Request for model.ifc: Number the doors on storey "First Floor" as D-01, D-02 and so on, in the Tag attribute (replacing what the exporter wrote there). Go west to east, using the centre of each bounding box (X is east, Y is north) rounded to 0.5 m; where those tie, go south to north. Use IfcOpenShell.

First a look at what the model holds.

```python
import ifcopenshell
import ifcopenshell.util.element
import ifcopenshell.util.placement

model = ifcopenshell.open("model.ifc")
print(model.schema)
storey = next(s for s in model.by_type("IfcBuildingStorey") if s.Name == "First Floor")
doors = [e for e in ifcopenshell.util.element.get_decomposition(storey) if e.is_a("IfcDoor")]
for e in sorted(doors, key=lambda e: e.id()):
    origin = ifcopenshell.util.placement.get_local_placement(e.ObjectPlacement)[:3, 3]
    print(e.id(), e.Tag, e.Name, origin.round(2) + 0.0, sep=" | ")
```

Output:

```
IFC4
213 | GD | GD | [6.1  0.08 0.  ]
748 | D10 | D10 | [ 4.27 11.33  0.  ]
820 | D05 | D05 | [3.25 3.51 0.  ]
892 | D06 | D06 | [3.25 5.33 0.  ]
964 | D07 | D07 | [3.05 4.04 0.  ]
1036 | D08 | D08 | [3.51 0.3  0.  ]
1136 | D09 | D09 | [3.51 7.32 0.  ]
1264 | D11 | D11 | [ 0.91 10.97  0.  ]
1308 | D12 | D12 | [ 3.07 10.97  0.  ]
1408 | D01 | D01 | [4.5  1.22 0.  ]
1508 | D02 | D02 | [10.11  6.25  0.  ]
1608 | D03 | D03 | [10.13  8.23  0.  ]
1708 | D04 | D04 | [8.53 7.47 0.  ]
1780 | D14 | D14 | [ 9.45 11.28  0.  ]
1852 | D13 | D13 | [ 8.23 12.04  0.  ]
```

```python
import ifcopenshell
import ifcopenshell.geom
import ifcopenshell.util.element
import ifcopenshell.util.shape

model = ifcopenshell.open("model.ifc")
settings = ifcopenshell.geom.settings()
settings.set("use-world-coords", True)


def centre(element):
    shape = ifcopenshell.geom.create_shape(settings, element)
    return ifcopenshell.util.shape.get_bbox_centroid(shape.geometry)


storey = next(s for s in model.by_type("IfcBuildingStorey") if s.Name == "First Floor")
doors = [e for e in ifcopenshell.util.element.get_decomposition(storey) if e.is_a("IfcDoor")]

# Insertion points can sit at a corner or the storey origin, so sort by the geometry (in metres).
centres = {e: centre(e) for e in doors}
doors.sort(key=lambda e: (round(centres[e][0] / 0.5), centres[e][1]))

for i, e in enumerate(doors, start=1):
    number = f"D-{i:02d}"
    e.Tag = number
    print(e.id(), number)

model.write("model_v2.ifc")
```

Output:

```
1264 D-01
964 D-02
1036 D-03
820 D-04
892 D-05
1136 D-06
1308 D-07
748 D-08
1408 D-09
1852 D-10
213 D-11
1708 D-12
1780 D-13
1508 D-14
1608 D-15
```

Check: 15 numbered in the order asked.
